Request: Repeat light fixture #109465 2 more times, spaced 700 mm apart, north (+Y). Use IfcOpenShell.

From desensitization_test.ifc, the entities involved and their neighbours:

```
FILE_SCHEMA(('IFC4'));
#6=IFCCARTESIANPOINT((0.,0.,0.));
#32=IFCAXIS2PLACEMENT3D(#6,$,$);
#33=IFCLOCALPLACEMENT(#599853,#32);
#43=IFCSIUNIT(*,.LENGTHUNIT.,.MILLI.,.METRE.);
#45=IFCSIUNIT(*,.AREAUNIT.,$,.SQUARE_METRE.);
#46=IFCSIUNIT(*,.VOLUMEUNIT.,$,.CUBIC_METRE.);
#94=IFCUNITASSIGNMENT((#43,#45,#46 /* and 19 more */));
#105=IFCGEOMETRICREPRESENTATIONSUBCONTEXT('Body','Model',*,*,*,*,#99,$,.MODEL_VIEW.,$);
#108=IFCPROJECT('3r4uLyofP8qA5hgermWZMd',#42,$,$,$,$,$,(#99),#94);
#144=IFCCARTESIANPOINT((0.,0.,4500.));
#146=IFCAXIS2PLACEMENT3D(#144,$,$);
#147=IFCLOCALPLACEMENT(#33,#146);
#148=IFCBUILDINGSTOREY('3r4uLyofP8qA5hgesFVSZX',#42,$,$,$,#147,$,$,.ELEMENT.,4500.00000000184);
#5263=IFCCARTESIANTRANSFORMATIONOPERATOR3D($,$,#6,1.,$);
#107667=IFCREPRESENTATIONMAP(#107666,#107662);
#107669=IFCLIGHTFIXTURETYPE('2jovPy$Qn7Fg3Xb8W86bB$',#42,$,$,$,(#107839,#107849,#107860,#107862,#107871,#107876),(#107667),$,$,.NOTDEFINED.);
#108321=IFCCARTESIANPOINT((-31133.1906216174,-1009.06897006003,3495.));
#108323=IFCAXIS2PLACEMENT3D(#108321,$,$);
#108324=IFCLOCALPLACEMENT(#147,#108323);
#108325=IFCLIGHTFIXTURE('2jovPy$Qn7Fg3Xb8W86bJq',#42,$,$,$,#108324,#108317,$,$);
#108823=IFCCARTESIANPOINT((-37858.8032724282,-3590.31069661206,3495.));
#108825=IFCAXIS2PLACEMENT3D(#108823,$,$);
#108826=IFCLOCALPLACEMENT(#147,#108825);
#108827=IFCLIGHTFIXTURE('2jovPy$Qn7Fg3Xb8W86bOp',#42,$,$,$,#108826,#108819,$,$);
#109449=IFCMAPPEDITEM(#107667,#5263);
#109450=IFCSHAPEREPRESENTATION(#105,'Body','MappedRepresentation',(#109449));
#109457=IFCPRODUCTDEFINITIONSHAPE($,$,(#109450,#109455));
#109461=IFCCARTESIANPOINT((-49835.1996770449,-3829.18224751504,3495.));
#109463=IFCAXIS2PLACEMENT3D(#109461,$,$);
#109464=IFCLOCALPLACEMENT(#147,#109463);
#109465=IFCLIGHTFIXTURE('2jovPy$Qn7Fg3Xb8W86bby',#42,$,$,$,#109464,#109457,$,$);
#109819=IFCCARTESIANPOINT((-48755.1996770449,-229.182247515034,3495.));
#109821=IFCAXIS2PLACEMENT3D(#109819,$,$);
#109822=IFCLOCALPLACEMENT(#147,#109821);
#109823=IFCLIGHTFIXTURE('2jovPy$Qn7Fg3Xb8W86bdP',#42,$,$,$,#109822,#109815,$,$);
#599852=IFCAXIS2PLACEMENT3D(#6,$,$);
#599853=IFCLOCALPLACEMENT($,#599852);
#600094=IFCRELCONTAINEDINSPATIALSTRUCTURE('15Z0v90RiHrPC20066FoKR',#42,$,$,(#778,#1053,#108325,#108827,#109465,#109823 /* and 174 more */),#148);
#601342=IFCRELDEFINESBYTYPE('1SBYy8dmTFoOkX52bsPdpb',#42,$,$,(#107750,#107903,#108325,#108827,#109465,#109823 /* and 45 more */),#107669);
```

```python
import numpy as np
import ifcopenshell
import ifcopenshell.api.geometry
import ifcopenshell.api.root
import ifcopenshell.util.element
import ifcopenshell.util.placement

model = ifcopenshell.open("desensitization_test.ifc")


def reuse_history(source, copy):
    """copy_class also copies each property set's owner history, people and application; keep the originals."""
    for rel in copy.IsDefinedBy:
        if rel.is_a("IfcRelDefinesByProperties") and (history := rel.RelatingPropertyDefinition.OwnerHistory):
            rel.RelatingPropertyDefinition.OwnerHistory = source.OwnerHistory
            ifcopenshell.util.element.remove_deep2(model, history)


source = model.by_guid("2jovPy$Qn7Fg3Xb8W86bby")
base = ifcopenshell.util.placement.get_local_placement(source.ObjectPlacement)
step = np.array([0.0, 1.0, 0.0]) * 700.0

for i in range(1, 3):
    copy = ifcopenshell.api.root.copy_class(model, product=source)
    copy.Representation = ifcopenshell.util.element.copy_deep(
        model, source.Representation, exclude=["IfcGeometricRepresentationContext", "IfcRepresentationMap"]
    )
    reuse_history(source, copy)
    matrix = base.copy()
    matrix[:3, 3] += i * step
    print("added at", matrix[:3, 3].round(3) + 0.0)
    ifcopenshell.api.geometry.edit_object_placement(model, product=copy, matrix=matrix, is_si=False)

model.write("desensitization_test_updated.ifc")
```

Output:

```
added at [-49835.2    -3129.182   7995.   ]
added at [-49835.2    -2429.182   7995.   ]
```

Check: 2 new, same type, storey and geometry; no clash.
